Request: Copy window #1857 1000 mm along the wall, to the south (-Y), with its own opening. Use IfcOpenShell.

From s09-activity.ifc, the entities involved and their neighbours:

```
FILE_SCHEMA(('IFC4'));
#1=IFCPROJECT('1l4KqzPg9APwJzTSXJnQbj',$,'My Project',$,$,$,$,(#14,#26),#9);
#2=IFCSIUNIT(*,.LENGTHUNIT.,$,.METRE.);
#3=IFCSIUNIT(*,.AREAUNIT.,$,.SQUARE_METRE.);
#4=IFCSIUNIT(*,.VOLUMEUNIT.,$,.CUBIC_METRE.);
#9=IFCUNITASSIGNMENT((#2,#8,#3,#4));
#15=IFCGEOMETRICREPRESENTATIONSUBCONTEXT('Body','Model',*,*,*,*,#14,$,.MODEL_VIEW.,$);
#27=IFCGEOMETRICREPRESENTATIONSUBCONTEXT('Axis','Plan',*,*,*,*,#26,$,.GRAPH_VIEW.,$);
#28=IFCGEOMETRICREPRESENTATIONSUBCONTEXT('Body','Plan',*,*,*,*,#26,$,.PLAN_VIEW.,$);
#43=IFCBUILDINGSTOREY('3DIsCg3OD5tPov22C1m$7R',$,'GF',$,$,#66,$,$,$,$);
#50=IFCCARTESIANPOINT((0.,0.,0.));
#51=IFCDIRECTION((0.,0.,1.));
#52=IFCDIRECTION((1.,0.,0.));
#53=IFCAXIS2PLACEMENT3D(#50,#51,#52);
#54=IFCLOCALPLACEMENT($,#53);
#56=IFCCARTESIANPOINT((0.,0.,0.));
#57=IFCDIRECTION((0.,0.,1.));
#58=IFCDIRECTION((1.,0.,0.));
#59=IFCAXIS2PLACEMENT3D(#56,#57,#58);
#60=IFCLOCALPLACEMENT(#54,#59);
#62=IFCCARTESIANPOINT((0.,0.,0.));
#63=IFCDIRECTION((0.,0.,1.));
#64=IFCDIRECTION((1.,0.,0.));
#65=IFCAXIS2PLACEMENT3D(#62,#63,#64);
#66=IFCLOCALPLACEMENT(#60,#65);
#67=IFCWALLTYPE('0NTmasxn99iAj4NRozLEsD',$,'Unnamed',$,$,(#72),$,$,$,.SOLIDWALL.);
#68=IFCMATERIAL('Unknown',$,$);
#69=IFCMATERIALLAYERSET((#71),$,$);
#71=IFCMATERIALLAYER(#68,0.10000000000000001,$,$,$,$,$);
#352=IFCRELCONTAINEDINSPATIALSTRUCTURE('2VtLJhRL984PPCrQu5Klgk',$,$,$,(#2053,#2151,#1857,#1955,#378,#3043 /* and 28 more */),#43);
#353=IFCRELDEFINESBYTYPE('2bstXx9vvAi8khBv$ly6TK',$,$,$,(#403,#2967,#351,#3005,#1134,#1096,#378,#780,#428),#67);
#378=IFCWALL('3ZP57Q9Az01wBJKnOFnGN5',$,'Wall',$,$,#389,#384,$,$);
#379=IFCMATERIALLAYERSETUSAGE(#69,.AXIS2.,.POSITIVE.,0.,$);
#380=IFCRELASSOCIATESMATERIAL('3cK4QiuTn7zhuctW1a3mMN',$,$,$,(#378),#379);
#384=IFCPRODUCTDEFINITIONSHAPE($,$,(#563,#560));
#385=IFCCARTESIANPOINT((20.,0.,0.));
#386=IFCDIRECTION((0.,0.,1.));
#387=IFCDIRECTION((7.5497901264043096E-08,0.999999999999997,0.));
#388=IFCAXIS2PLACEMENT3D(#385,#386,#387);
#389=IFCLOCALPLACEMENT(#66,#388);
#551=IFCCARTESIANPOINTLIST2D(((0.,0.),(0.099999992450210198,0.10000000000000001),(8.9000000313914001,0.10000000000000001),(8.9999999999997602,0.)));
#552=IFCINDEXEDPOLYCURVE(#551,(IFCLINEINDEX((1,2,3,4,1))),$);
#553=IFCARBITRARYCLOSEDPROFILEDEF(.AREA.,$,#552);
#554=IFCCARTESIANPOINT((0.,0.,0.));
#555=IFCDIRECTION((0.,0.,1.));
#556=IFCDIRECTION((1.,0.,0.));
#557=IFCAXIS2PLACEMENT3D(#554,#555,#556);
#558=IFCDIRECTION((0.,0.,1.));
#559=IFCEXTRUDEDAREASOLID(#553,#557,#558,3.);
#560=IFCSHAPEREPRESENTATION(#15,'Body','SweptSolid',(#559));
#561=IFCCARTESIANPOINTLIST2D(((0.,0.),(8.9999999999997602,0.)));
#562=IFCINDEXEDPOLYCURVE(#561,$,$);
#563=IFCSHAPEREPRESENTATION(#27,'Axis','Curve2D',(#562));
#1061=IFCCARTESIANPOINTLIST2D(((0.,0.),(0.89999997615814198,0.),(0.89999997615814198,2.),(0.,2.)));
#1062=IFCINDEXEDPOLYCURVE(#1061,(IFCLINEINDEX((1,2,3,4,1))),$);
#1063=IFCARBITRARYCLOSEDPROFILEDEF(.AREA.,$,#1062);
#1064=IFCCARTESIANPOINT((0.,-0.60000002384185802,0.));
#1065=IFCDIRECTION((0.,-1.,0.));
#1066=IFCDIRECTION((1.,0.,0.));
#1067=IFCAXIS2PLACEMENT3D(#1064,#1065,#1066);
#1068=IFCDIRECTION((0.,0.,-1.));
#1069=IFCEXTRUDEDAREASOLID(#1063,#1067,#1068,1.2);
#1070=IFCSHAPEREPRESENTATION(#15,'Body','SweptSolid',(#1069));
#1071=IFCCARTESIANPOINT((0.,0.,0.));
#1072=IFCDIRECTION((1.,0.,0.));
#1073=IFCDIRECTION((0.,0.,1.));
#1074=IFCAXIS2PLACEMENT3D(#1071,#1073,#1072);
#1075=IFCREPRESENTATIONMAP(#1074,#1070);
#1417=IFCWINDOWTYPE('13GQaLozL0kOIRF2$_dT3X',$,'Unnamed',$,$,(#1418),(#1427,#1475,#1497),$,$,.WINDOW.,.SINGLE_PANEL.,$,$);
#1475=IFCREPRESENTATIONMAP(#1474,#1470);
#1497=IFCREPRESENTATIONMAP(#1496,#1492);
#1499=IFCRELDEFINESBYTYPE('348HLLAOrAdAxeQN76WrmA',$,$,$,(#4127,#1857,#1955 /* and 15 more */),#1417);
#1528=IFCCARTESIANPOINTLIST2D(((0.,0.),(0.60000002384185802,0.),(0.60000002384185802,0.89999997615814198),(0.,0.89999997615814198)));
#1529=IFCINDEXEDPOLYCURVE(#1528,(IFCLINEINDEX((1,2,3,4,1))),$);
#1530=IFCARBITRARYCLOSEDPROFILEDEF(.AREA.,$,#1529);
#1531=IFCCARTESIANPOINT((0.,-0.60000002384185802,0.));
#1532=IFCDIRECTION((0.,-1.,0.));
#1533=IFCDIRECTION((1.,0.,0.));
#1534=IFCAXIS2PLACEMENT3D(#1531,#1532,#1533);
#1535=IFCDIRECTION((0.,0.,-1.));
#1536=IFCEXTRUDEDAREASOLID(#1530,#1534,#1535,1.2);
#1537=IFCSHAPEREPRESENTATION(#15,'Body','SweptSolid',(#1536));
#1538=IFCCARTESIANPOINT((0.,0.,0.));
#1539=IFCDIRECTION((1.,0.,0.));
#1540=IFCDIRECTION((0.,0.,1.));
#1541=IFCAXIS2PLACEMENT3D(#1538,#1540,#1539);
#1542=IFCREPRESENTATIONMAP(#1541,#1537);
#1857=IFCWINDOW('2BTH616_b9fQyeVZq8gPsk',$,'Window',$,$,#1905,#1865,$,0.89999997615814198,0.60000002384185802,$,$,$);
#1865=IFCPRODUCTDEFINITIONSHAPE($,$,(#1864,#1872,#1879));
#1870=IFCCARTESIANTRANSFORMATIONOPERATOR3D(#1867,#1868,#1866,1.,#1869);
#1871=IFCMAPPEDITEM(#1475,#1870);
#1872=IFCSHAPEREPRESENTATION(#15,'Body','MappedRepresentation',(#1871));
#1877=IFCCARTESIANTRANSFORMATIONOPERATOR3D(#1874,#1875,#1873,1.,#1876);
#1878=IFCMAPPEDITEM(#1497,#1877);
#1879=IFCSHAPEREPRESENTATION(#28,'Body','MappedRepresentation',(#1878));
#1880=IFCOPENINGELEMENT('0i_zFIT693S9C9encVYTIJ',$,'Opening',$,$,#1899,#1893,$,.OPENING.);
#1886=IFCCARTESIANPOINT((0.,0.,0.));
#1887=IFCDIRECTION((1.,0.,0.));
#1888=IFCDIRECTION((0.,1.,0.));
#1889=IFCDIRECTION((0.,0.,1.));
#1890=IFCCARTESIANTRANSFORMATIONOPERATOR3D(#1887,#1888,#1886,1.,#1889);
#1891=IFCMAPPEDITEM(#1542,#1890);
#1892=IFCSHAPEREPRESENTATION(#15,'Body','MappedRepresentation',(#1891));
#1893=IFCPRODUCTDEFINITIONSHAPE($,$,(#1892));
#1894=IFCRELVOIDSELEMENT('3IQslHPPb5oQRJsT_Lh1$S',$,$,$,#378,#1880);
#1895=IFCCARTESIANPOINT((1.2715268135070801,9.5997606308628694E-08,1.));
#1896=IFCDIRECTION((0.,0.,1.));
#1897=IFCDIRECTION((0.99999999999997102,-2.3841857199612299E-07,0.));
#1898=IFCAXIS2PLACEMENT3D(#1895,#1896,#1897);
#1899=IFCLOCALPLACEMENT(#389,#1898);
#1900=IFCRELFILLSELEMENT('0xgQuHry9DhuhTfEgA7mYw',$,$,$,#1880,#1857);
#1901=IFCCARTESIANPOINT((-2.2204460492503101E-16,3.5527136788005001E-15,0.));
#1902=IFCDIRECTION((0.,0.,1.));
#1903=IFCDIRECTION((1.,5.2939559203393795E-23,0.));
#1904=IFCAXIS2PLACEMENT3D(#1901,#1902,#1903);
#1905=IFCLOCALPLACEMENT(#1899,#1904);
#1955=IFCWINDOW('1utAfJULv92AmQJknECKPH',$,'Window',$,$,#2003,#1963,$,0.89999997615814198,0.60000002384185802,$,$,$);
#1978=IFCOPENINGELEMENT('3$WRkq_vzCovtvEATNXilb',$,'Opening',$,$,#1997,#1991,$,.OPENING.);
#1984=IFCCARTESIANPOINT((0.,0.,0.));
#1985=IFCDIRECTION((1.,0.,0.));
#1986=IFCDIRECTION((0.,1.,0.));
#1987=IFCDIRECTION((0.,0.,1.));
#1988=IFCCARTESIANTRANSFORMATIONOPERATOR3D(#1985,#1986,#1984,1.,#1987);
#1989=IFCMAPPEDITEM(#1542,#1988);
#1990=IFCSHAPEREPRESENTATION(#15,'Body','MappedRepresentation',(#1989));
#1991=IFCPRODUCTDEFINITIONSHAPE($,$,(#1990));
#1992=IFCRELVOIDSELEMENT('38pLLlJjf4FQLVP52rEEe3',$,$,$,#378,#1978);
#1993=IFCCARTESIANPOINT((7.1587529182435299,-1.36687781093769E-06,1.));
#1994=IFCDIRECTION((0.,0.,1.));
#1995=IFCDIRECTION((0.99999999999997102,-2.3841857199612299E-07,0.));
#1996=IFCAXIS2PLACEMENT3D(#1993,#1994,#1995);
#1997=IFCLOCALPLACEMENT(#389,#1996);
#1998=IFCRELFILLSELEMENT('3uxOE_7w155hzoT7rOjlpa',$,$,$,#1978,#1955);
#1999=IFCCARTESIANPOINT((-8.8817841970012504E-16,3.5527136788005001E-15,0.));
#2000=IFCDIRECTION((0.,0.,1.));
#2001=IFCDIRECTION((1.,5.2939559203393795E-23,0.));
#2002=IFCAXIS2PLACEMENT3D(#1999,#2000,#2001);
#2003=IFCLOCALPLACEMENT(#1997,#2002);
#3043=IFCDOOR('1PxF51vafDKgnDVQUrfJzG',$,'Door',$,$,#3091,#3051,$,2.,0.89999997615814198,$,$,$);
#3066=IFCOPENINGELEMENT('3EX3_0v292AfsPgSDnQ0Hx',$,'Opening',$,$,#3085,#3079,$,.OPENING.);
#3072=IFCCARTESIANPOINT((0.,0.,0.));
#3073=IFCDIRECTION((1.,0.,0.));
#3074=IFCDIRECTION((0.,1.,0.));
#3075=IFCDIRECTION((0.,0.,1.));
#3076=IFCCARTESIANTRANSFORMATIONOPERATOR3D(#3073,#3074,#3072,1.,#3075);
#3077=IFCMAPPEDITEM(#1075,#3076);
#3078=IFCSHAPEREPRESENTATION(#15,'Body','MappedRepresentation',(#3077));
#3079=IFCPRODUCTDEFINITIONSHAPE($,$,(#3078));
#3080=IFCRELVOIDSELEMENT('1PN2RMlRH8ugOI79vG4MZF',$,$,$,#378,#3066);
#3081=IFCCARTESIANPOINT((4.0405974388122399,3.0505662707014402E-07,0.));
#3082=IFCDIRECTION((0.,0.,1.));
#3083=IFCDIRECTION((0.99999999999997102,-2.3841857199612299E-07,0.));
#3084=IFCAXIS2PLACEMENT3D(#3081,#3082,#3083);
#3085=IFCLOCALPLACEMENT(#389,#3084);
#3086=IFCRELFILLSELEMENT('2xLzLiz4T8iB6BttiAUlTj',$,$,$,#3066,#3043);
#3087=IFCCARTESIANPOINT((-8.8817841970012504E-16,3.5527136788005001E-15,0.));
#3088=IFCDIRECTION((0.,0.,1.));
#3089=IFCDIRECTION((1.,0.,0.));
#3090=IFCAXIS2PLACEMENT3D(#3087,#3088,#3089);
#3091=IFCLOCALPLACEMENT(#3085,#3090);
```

```python
import ifcopenshell
import ifcopenshell.api.feature
import ifcopenshell.api.geometry
import ifcopenshell.api.root
import ifcopenshell.geom
import ifcopenshell.util.element
import ifcopenshell.util.placement
import ifcopenshell.util.shape
import ifcopenshell.util.unit

model = ifcopenshell.open("s09-activity.ifc")
unit_scale = ifcopenshell.util.unit.calculate_unit_scale(model)
settings = ifcopenshell.geom.settings()


def volume(element):
    """Net volume in cubic metres, openings subtracted."""
    shape = ifcopenshell.geom.create_shape(settings, element)
    return ifcopenshell.util.shape.get_volume(shape.geometry)


window = model.by_id(1857)
opening = window.FillsVoids[0].RelatingOpeningElement
wall = opening.VoidsElements[0].RelatingBuildingElement
before = volume(wall)
shift = ifcopenshell.util.placement.get_local_placement(wall.ObjectPlacement)[:3, 0] * -1 / unit_scale

# copy_class copies the void relationship, type, container and properties, but no geometry.
new_opening = ifcopenshell.api.root.copy_class(model, product=opening)
new_opening.Representation = ifcopenshell.util.element.copy_deep(
    model, opening.Representation, exclude=["IfcGeometricRepresentationContext", "IfcRepresentationMap"]
)
new_window = ifcopenshell.api.root.copy_class(model, product=window)
new_window.Representation = ifcopenshell.util.element.copy_deep(
    model, window.Representation, exclude=["IfcGeometricRepresentationContext", "IfcRepresentationMap"]
)
ifcopenshell.api.feature.add_filling(model, opening=new_opening, element=new_window)

for old, new in ((opening, new_opening), (window, new_window)):
    matrix = ifcopenshell.util.placement.get_local_placement(old.ObjectPlacement)
    matrix[:3, 3] += shift
    ifcopenshell.api.geometry.edit_object_placement(model, product=new, matrix=matrix, is_si=False)

after = volume(wall)

print(f"wall volume {before:.3f} -> {after:.3f} m3")

model.write("s09-activity-out.ifc")
```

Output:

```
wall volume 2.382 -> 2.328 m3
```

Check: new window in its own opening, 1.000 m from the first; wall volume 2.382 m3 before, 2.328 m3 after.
